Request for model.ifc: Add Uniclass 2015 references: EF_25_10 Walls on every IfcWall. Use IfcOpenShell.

First a look at what the model holds.

```python
import ifcopenshell

model = ifcopenshell.open("model.ifc")
print(model.schema)
print("classifications:", [c.Name for c in model.by_type("IfcClassification")])
for ifc_class in ("IfcDoor", "IfcRoof", "IfcStair", "IfcWall", "IfcWindow"):
    print(ifc_class, len(model.by_type(ifc_class)))
```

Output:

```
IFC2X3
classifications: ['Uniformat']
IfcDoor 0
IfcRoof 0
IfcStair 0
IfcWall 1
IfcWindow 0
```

```python
import ifcopenshell
import ifcopenshell.api.classification

model = ifcopenshell.open("model.ifc")

# IFC2X3 requires Source and Edition and has no link from the project to the system.
system = model.create_entity("IfcClassification", Source="NBS", Edition="2015", Name="Uniclass 2015")

codes = {
    "IfcWall": ("EF_25_10", "Walls"),
}
for ifc_class, (code, name) in codes.items():
    products = model.by_type(ifc_class)
    ifcopenshell.api.classification.add_reference(
        model, products=products, classification=system, identification=code, name=name
    )
    print(code, len(products))

model.write("model-out.ifc")
```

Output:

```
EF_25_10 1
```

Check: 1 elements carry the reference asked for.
